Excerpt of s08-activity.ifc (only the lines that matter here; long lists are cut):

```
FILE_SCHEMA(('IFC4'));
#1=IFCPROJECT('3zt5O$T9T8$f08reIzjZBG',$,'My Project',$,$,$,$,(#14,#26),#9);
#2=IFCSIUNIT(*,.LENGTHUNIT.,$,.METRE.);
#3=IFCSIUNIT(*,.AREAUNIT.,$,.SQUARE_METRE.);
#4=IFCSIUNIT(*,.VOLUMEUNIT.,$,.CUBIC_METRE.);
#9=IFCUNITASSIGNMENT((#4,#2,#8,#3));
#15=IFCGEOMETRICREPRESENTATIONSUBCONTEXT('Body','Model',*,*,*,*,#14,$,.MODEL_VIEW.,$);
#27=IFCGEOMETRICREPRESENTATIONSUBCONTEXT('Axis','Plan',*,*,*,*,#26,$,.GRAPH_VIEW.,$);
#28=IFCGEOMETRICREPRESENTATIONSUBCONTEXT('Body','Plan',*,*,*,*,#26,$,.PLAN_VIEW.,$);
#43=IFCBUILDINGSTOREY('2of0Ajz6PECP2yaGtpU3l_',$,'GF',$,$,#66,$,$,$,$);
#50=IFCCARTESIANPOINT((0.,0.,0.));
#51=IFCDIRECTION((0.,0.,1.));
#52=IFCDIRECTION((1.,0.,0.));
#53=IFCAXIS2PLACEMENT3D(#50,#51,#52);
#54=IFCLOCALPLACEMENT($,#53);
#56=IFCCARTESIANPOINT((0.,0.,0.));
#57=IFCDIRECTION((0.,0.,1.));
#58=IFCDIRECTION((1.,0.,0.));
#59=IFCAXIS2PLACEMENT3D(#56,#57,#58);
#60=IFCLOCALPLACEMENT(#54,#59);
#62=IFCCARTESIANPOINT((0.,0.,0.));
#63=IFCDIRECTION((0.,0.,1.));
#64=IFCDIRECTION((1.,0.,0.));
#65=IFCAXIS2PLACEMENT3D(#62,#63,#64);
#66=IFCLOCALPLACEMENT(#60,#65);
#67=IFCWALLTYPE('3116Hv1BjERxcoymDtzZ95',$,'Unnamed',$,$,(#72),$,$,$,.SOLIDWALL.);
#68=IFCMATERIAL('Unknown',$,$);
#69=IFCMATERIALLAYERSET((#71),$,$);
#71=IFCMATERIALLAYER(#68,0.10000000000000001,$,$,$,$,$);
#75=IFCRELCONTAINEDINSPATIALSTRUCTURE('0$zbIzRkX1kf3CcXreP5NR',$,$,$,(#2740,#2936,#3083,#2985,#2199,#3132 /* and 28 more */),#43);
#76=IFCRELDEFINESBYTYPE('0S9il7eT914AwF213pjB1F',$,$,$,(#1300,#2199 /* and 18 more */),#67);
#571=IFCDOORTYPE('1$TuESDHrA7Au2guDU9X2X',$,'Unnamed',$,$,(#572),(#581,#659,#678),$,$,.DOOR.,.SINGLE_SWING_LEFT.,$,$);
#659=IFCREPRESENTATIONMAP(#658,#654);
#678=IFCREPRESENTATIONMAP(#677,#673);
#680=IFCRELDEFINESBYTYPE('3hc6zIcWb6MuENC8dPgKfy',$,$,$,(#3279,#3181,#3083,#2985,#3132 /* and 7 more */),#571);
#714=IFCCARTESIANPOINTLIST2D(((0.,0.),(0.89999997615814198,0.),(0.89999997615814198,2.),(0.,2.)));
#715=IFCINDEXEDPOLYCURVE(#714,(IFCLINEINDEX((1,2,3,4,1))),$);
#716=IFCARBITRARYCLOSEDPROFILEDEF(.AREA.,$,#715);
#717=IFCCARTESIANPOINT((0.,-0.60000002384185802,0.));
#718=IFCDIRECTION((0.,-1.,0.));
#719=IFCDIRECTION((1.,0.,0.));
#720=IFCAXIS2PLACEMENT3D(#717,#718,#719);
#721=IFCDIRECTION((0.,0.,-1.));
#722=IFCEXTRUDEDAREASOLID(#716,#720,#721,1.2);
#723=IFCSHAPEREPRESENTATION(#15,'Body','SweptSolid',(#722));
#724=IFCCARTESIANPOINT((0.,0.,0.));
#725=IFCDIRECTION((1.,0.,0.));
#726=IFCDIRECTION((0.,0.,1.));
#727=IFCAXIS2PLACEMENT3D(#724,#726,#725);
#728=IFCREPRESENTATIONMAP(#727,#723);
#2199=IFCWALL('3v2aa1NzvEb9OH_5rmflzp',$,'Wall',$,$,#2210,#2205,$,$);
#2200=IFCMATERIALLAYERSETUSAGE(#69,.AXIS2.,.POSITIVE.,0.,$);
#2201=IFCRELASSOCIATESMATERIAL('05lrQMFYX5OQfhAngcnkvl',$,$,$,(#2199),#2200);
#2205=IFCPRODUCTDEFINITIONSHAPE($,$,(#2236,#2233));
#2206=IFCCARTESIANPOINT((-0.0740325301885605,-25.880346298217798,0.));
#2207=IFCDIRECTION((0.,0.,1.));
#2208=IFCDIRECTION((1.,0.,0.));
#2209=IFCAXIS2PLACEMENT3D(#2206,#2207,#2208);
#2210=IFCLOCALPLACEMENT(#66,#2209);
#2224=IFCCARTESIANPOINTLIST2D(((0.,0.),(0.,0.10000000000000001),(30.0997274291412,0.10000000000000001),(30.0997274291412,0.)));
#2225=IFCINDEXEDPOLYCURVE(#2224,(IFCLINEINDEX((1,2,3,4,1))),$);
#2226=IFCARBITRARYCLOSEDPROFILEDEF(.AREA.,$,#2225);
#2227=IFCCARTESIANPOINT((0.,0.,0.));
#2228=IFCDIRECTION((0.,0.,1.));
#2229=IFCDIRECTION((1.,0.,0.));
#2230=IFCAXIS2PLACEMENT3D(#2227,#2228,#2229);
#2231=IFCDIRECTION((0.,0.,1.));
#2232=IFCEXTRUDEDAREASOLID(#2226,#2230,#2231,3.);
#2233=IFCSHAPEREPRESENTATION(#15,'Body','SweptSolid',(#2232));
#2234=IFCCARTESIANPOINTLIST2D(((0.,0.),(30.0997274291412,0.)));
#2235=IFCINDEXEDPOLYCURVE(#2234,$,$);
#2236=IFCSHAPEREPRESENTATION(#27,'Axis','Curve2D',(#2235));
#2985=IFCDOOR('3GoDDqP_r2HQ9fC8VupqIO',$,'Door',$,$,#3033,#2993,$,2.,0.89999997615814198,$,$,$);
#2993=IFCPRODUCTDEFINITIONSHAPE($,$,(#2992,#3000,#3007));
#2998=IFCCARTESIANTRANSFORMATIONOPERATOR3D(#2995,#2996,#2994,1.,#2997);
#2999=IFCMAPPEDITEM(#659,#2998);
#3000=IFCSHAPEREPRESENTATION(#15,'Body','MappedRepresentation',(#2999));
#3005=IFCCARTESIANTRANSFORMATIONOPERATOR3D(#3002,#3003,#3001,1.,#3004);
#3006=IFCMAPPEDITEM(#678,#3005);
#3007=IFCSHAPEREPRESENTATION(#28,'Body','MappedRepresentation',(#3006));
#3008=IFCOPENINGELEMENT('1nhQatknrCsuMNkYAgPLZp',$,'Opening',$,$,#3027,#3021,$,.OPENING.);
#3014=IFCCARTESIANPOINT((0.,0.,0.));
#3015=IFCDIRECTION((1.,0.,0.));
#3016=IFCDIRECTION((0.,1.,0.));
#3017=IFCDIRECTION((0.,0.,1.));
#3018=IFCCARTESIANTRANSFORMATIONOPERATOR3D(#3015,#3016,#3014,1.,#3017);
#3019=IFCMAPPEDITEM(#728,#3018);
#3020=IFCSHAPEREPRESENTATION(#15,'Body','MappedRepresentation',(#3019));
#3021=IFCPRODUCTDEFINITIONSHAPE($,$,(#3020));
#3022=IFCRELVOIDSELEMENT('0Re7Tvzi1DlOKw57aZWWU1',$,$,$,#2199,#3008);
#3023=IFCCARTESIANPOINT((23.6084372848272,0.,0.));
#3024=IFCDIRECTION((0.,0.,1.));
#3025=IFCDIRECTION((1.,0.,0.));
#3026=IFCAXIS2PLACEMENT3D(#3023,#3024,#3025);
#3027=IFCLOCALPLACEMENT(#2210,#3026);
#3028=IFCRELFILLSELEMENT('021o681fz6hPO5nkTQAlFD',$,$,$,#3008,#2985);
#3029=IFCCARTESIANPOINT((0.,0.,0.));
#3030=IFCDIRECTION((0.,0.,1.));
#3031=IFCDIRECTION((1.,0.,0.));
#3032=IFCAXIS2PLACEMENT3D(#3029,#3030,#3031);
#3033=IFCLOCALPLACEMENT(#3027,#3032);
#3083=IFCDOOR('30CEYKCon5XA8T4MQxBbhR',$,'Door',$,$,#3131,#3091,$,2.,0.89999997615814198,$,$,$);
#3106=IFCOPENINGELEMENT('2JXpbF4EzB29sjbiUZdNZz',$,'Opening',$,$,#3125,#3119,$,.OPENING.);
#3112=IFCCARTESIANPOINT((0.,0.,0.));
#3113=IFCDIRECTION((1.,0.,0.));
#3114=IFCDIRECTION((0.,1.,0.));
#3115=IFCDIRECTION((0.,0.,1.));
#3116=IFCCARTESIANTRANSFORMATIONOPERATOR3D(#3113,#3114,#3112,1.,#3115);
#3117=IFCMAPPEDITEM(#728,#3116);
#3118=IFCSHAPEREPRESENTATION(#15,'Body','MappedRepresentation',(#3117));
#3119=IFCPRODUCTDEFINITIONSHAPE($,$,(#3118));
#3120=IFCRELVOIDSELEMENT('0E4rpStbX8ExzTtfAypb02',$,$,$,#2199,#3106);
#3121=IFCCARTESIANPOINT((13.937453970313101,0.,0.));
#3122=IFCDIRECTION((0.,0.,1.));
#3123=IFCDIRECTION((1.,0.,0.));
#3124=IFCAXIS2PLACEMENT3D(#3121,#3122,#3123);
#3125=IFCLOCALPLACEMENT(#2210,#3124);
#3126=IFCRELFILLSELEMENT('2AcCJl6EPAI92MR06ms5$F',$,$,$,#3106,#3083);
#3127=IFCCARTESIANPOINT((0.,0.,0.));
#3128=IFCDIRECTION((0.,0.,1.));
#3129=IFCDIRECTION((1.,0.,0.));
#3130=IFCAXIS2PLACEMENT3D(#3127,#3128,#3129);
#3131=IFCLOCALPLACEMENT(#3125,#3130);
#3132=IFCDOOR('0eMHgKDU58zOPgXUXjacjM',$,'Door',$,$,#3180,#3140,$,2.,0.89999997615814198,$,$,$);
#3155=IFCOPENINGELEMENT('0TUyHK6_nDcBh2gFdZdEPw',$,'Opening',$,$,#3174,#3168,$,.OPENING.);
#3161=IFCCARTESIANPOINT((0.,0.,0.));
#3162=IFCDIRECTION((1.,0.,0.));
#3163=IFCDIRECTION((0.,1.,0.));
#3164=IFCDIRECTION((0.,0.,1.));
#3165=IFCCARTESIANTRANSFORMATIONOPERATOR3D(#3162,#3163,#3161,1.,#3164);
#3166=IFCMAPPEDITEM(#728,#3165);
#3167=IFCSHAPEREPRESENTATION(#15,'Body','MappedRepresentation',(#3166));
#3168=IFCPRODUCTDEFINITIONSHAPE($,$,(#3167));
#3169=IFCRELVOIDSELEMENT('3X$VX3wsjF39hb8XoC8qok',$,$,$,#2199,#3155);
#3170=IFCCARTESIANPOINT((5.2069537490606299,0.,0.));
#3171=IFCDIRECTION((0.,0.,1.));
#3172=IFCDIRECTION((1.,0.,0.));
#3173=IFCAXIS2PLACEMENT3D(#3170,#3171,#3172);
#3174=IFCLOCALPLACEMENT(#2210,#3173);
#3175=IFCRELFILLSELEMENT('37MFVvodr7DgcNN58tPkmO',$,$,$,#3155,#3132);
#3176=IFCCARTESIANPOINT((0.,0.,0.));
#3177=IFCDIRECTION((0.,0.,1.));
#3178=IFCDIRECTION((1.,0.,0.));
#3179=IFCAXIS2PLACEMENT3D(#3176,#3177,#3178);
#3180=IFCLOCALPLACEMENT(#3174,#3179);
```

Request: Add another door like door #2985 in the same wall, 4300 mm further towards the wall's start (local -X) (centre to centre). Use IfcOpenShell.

```python
import ifcopenshell
import ifcopenshell.api.feature
import ifcopenshell.api.geometry
import ifcopenshell.api.root
import ifcopenshell.geom
import ifcopenshell.util.element
import ifcopenshell.util.placement
import ifcopenshell.util.shape
import ifcopenshell.util.unit

model = ifcopenshell.open("s08-activity.ifc")
unit_scale = ifcopenshell.util.unit.calculate_unit_scale(model)
settings = ifcopenshell.geom.settings()


def volume(element):
    """Net volume in cubic metres, openings subtracted."""
    shape = ifcopenshell.geom.create_shape(settings, element)
    return ifcopenshell.util.shape.get_volume(shape.geometry)


door = model.by_guid("3GoDDqP_r2HQ9fC8VupqIO")
opening = door.FillsVoids[0].RelatingOpeningElement
wall = opening.VoidsElements[0].RelatingBuildingElement
before = volume(wall)
shift = ifcopenshell.util.placement.get_local_placement(wall.ObjectPlacement)[:3, 0] * -4.3 / unit_scale

# copy_class copies the void relationship, type, container and properties, but no geometry.
new_opening = ifcopenshell.api.root.copy_class(model, product=opening)
new_opening.Representation = ifcopenshell.util.element.copy_deep(
    model, opening.Representation, exclude=["IfcGeometricRepresentationContext", "IfcRepresentationMap"]
)
new_door = ifcopenshell.api.root.copy_class(model, product=door)
new_door.Representation = ifcopenshell.util.element.copy_deep(
    model, door.Representation, exclude=["IfcGeometricRepresentationContext", "IfcRepresentationMap"]
)
ifcopenshell.api.feature.add_filling(model, opening=new_opening, element=new_door)

for old, new in ((opening, new_opening), (door, new_door)):
    matrix = ifcopenshell.util.placement.get_local_placement(old.ObjectPlacement)
    matrix[:3, 3] += shift
    ifcopenshell.api.geometry.edit_object_placement(model, product=new, matrix=matrix, is_si=False)

after = volume(wall)

print(f"wall volume {before:.3f} -> {after:.3f} m3")

model.write("s08-activity_rev.ifc")
```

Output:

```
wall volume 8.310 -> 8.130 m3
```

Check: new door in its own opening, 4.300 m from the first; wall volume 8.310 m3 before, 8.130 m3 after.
